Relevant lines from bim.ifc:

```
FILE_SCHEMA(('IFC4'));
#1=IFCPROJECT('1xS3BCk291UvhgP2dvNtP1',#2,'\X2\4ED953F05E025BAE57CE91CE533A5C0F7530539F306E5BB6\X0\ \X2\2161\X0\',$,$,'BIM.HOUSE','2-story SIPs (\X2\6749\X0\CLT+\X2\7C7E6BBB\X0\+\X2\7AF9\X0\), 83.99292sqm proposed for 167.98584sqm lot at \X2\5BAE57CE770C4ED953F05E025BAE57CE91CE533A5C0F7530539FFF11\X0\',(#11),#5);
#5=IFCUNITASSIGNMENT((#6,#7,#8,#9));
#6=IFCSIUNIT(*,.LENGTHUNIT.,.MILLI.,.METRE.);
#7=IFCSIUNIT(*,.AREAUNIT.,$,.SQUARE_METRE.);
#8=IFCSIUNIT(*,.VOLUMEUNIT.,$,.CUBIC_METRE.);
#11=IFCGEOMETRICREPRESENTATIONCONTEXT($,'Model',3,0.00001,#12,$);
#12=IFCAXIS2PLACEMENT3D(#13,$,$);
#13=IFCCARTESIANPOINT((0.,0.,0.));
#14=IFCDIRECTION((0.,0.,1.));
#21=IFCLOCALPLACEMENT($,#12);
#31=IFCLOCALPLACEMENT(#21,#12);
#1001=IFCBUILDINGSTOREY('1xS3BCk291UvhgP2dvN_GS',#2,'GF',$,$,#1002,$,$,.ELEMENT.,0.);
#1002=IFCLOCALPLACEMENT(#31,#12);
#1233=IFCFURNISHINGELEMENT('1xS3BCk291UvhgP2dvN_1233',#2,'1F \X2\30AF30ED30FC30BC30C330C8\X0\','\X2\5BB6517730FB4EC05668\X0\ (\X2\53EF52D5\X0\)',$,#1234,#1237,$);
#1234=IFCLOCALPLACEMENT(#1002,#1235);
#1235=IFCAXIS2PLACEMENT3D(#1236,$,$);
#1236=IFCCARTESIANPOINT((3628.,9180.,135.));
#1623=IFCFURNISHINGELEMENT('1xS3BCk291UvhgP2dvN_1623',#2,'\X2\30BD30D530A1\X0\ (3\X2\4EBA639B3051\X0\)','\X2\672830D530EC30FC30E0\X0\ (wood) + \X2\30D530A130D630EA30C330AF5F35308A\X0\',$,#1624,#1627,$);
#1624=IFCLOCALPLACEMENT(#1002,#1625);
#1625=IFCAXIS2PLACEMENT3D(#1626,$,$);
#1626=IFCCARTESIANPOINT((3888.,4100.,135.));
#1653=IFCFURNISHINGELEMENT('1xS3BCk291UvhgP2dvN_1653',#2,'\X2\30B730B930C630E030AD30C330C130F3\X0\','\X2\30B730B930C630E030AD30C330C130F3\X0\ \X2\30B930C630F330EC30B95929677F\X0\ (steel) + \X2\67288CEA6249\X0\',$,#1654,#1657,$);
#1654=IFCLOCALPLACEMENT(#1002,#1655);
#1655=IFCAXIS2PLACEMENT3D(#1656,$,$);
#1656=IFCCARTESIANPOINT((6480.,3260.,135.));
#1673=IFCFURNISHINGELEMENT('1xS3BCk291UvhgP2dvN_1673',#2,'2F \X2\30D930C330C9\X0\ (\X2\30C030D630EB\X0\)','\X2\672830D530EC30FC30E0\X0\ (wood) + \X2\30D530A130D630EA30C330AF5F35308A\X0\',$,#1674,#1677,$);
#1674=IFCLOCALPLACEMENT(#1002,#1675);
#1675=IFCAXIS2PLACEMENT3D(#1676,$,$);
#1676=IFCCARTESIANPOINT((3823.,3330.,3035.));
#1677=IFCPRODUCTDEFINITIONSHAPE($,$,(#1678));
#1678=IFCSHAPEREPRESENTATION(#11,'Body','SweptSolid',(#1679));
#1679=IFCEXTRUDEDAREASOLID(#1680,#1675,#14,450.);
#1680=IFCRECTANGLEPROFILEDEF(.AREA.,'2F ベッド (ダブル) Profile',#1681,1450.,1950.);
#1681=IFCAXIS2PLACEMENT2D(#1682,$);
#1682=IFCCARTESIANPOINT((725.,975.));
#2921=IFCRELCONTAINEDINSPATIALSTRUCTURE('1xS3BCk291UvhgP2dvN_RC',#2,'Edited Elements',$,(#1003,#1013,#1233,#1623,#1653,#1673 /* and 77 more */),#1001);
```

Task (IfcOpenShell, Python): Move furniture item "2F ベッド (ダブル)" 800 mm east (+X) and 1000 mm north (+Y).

```python
import ifcopenshell
import ifcopenshell.api.geometry
import ifcopenshell.util.placement

model = ifcopenshell.open("bim.ifc")

item = model.by_guid("1xS3BCk291UvhgP2dvN_1673")
matrix = ifcopenshell.util.placement.get_local_placement(item.ObjectPlacement)
matrix[0, 3] += 800.0
matrix[1, 3] += 1000.0
ifcopenshell.api.geometry.edit_object_placement(model, product=item, matrix=matrix, is_si=False)

print(ifcopenshell.util.placement.get_local_placement(item.ObjectPlacement).round(3) + 0.0)

model.write("bim_v2.ifc")
```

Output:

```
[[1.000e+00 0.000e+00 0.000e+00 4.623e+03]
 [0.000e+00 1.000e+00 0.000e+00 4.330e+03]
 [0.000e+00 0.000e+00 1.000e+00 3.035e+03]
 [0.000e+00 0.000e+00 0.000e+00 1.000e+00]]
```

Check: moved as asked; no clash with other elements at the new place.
